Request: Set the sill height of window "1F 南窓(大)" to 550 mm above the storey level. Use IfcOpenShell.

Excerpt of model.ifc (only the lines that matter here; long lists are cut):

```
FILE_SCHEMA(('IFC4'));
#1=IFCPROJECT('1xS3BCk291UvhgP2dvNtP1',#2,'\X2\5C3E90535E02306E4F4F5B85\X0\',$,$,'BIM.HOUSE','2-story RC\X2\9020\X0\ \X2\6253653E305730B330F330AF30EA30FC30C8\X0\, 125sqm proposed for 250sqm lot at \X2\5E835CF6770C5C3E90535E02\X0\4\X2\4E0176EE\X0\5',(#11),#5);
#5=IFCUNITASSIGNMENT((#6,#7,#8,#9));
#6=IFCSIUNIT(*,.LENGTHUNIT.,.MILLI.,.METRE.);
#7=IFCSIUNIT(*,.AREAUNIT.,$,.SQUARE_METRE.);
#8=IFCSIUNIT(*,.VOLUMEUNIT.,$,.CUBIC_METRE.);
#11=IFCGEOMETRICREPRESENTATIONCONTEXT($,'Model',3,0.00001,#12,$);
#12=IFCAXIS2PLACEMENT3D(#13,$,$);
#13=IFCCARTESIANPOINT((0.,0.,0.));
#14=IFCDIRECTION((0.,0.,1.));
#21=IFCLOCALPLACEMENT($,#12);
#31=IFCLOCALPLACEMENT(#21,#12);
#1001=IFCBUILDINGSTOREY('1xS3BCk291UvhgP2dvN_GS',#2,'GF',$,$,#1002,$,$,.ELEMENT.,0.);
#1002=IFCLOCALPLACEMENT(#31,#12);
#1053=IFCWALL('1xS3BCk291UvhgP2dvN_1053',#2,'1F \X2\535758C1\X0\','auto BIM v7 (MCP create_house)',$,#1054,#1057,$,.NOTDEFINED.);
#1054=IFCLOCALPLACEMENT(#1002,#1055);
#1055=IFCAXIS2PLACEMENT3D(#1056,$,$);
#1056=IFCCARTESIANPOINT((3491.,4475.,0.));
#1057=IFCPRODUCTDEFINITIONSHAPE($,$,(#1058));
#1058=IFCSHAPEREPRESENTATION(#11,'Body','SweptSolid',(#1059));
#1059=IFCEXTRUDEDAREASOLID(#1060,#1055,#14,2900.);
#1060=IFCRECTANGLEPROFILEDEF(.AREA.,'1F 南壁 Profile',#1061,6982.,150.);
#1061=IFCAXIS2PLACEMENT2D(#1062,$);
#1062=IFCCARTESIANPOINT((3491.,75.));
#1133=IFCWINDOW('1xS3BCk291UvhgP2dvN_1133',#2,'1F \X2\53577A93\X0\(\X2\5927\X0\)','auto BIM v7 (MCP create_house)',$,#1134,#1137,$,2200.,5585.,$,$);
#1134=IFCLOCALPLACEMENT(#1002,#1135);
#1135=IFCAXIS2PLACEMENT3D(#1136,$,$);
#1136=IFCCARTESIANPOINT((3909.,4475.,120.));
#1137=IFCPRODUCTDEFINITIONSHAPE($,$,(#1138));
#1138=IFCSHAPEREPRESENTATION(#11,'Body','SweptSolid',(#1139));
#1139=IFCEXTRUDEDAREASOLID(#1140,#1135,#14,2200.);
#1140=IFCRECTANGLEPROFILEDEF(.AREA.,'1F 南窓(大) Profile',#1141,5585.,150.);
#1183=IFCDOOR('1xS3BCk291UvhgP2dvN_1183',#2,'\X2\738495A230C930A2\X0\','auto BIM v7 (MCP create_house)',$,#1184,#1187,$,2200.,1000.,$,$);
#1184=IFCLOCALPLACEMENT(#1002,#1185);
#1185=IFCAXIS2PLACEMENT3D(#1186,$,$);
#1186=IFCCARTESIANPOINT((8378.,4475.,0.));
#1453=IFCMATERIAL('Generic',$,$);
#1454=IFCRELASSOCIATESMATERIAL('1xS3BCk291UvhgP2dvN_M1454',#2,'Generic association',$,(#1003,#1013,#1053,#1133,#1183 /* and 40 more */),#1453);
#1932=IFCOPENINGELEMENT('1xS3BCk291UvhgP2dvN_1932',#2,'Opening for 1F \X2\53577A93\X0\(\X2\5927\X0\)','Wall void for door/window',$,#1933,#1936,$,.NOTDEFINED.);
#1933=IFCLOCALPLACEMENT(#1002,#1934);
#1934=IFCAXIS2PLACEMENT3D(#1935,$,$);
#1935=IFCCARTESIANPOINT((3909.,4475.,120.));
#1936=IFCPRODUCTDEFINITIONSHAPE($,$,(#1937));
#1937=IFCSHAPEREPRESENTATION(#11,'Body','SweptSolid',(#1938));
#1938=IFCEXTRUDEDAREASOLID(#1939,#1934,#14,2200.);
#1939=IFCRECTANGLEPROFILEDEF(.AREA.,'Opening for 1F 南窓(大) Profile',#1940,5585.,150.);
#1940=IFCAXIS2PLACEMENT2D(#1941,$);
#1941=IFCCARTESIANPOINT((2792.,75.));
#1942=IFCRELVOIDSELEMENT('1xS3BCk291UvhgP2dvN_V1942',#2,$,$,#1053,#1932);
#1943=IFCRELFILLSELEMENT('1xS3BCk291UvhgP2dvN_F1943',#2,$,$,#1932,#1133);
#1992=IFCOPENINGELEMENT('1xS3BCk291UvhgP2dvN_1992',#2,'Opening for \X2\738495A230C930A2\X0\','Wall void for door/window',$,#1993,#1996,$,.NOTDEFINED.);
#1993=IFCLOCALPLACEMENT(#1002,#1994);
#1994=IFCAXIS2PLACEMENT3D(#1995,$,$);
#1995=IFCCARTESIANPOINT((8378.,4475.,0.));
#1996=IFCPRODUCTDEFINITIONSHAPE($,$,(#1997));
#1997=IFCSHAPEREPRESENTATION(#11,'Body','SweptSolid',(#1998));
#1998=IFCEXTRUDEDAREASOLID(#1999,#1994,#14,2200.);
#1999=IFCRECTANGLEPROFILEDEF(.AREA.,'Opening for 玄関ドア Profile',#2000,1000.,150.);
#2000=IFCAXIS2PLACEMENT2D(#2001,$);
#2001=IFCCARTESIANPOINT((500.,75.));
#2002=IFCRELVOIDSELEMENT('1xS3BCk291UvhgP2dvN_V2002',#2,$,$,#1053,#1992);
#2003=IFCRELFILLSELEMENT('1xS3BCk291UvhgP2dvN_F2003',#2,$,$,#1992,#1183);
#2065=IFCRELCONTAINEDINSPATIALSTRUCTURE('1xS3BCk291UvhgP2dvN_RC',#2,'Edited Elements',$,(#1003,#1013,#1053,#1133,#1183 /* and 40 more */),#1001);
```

```python
import numpy as np
import ifcopenshell
import ifcopenshell.api.geometry
import ifcopenshell.geom
import ifcopenshell.util.element
import ifcopenshell.util.placement
import ifcopenshell.util.shape
import ifcopenshell.util.unit

model = ifcopenshell.open("model.ifc")
unit_scale = ifcopenshell.util.unit.calculate_unit_scale(model)

window = model.by_id(1133)
opening = window.FillsVoids[0].RelatingOpeningElement
storey = ifcopenshell.util.element.get_container(window, ifc_class="IfcBuildingStorey")
level = ifcopenshell.util.placement.get_local_placement(storey.ObjectPlacement)[2, 3]

# The opening's origin need not be at the sill, so measure its lowest point.
shape = ifcopenshell.geom.create_shape(ifcopenshell.geom.settings(), opening)
bottom = ifcopenshell.util.shape.get_shape_bottom_elevation(shape, shape.geometry) / unit_scale
dz = level + 550.0 - bottom

shift = np.array([0.0, 0.0, dz])
# The window is not placed relative to its opening, so move both.
for product in (opening, window):
    matrix = ifcopenshell.util.placement.get_local_placement(product.ObjectPlacement)
    matrix[:3, 3] += shift
    ifcopenshell.api.geometry.edit_object_placement(model, product=product, matrix=matrix, is_si=False)

print(f"moved by {dz * unit_scale:+.3f} m")

model.write("model-out.ifc")
```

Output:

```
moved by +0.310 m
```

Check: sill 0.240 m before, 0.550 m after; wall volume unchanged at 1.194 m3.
